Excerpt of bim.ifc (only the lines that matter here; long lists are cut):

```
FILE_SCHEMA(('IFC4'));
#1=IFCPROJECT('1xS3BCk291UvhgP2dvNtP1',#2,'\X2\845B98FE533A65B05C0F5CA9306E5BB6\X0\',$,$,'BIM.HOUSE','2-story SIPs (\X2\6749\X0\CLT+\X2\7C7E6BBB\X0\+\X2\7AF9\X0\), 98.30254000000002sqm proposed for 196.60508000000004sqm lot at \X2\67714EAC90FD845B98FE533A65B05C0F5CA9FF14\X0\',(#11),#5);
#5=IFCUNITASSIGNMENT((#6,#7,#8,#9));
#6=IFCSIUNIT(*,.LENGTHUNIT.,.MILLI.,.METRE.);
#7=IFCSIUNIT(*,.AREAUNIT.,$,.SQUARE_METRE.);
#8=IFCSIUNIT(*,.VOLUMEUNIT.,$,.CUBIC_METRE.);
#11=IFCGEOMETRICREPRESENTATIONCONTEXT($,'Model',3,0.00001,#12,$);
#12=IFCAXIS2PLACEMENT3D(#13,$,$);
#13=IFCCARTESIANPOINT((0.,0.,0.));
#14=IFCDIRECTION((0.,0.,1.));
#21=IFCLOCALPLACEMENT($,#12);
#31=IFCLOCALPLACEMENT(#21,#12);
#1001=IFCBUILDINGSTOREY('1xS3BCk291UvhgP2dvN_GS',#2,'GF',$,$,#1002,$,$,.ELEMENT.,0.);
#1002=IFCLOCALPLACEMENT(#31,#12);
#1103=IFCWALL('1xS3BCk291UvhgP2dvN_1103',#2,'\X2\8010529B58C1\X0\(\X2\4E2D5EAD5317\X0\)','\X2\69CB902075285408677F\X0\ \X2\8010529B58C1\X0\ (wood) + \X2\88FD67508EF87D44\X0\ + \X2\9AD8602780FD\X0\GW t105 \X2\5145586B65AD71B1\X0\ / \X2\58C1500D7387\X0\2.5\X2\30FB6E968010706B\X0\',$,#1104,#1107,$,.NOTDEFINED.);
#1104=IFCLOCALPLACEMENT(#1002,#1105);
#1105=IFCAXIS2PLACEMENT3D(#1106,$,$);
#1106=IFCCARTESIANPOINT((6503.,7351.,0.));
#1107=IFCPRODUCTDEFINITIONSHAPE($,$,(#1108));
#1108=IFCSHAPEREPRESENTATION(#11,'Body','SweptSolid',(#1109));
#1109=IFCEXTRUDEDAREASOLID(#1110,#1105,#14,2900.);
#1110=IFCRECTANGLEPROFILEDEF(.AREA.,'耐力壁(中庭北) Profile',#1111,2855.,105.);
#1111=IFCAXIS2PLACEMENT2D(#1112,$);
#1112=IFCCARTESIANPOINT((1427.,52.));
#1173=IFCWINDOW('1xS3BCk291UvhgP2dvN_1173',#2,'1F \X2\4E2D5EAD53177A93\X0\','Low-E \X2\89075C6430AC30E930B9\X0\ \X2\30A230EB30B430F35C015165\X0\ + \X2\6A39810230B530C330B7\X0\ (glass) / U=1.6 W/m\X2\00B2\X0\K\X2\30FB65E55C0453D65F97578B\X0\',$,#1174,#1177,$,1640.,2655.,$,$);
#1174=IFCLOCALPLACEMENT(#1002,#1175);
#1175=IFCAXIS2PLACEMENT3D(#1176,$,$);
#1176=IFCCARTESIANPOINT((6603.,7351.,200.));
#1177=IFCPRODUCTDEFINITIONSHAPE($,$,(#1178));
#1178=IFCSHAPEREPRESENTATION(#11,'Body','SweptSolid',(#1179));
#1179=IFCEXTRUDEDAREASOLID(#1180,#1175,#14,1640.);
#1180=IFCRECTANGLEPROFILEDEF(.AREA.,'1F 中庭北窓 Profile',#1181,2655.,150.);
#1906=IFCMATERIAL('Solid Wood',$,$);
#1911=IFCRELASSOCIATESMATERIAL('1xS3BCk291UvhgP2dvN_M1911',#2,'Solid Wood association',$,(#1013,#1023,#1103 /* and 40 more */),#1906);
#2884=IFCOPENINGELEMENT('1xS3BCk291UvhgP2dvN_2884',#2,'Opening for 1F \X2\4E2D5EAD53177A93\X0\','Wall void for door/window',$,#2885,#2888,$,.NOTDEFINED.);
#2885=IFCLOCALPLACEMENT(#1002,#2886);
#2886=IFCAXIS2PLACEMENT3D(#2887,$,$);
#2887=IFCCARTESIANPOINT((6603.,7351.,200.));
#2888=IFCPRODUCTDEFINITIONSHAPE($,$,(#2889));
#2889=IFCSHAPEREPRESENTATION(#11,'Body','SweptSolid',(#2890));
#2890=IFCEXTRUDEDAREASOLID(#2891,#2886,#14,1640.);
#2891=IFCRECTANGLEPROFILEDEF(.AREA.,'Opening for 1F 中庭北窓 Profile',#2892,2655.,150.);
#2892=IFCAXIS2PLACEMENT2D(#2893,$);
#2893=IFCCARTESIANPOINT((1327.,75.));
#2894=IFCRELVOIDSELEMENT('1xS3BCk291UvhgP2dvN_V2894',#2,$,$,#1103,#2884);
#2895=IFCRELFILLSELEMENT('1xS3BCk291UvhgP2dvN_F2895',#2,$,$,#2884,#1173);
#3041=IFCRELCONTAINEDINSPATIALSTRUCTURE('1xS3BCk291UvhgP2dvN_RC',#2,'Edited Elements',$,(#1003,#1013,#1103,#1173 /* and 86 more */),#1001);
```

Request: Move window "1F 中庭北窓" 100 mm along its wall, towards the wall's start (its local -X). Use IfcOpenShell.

```python
import ifcopenshell
import ifcopenshell.api.geometry
import ifcopenshell.util.placement
import ifcopenshell.util.unit

model = ifcopenshell.open("bim.ifc")
unit_scale = ifcopenshell.util.unit.calculate_unit_scale(model)

window = model.by_guid("1xS3BCk291UvhgP2dvN_1173")
opening = window.FillsVoids[0].RelatingOpeningElement
wall = opening.VoidsElements[0].RelatingBuildingElement

wall_matrix = ifcopenshell.util.placement.get_local_placement(wall.ObjectPlacement)
shift = wall_matrix[:3, 0] * -0.1 / unit_scale
before = ifcopenshell.util.placement.get_local_placement(window.ObjectPlacement)[:3, 3].copy()

# The window is not placed relative to its opening, so move both.
for product in (opening, window):
    matrix = ifcopenshell.util.placement.get_local_placement(product.ObjectPlacement)
    matrix[:3, 3] += shift
    ifcopenshell.api.geometry.edit_object_placement(model, product=product, matrix=matrix, is_si=False)

after = ifcopenshell.util.placement.get_local_placement(window.ObjectPlacement)[:3, 3]
print("window moved by", (after - before).round(3) + 0.0)

model.write("bim_v2.ifc")
```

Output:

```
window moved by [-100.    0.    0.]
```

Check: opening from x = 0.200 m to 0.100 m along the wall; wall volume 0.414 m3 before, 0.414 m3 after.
